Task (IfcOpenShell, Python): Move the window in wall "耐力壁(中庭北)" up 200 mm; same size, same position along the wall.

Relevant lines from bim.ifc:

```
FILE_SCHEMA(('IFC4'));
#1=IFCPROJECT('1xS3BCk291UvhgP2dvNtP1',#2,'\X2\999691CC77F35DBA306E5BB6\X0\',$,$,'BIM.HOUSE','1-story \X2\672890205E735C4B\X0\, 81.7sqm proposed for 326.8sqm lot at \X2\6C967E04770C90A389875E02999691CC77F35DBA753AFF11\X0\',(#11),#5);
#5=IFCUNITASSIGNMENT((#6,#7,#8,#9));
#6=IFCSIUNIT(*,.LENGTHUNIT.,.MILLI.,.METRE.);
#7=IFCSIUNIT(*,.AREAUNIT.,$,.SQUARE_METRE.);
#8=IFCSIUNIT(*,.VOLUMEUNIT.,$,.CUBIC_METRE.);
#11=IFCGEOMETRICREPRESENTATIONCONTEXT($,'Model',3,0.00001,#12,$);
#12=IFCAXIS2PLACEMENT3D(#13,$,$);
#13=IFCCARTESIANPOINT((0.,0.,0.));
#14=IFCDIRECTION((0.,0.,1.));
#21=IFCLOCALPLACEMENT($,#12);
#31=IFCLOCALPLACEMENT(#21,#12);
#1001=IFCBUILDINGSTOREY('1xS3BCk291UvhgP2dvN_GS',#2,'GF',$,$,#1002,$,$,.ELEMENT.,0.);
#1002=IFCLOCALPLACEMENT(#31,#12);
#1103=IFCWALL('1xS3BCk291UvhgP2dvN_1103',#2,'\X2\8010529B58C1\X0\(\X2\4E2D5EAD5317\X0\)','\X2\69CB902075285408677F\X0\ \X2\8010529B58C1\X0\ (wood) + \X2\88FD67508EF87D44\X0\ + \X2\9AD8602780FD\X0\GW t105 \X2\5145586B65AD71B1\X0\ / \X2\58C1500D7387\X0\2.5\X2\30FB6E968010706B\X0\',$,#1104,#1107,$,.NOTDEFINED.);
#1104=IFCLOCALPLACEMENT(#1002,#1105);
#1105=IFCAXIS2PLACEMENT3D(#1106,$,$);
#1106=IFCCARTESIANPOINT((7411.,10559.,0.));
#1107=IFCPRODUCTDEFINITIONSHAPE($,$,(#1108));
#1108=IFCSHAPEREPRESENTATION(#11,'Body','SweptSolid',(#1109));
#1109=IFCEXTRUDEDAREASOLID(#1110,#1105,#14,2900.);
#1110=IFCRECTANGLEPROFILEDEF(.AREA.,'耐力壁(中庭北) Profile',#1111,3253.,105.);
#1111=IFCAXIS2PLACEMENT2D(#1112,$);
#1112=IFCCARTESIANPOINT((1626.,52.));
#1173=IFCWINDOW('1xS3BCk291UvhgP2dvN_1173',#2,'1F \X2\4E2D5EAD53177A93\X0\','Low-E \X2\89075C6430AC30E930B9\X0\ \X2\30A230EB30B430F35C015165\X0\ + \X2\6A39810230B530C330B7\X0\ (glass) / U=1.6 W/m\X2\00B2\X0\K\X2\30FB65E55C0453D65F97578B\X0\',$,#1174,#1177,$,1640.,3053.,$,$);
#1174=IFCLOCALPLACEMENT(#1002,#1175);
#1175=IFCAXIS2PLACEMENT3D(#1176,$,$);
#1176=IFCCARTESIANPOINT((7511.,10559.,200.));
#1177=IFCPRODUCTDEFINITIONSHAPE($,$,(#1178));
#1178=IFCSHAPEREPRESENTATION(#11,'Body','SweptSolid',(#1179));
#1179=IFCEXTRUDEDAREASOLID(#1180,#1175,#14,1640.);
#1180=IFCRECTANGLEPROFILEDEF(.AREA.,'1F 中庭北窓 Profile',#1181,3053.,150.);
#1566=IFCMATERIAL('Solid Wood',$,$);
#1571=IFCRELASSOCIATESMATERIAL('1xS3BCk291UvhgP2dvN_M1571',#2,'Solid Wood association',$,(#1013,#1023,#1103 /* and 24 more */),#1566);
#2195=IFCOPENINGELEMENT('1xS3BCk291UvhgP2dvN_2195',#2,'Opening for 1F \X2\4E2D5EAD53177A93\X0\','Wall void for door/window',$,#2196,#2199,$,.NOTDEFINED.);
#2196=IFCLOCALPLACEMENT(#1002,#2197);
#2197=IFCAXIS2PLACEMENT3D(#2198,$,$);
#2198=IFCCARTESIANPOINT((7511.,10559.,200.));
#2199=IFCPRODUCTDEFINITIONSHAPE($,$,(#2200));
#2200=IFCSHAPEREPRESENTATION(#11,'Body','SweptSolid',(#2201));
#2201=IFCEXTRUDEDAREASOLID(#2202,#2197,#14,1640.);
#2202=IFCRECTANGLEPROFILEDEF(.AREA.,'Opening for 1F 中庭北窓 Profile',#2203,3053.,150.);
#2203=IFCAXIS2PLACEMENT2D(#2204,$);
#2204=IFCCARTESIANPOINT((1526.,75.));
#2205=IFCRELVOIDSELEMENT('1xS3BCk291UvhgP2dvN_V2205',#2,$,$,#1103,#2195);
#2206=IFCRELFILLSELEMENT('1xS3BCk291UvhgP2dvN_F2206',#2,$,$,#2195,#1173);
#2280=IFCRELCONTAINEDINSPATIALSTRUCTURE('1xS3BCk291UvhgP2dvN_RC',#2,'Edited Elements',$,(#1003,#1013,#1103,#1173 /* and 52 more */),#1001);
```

```python
import numpy as np
import ifcopenshell
import ifcopenshell.api.geometry
import ifcopenshell.util.placement
import ifcopenshell.util.unit

model = ifcopenshell.open("bim.ifc")
unit_scale = ifcopenshell.util.unit.calculate_unit_scale(model)

window = model.by_guid("1xS3BCk291UvhgP2dvN_1173")
opening = window.FillsVoids[0].RelatingOpeningElement
dz = 200.0

shift = np.array([0.0, 0.0, dz])
# The window is not placed relative to its opening, so move both.
for product in (opening, window):
    matrix = ifcopenshell.util.placement.get_local_placement(product.ObjectPlacement)
    matrix[:3, 3] += shift
    ifcopenshell.api.geometry.edit_object_placement(model, product=product, matrix=matrix, is_si=False)

print(f"moved by {dz * unit_scale:+.3f} m")

model.write("bim_edited.ifc")
```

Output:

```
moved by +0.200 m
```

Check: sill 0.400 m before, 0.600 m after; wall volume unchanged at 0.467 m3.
